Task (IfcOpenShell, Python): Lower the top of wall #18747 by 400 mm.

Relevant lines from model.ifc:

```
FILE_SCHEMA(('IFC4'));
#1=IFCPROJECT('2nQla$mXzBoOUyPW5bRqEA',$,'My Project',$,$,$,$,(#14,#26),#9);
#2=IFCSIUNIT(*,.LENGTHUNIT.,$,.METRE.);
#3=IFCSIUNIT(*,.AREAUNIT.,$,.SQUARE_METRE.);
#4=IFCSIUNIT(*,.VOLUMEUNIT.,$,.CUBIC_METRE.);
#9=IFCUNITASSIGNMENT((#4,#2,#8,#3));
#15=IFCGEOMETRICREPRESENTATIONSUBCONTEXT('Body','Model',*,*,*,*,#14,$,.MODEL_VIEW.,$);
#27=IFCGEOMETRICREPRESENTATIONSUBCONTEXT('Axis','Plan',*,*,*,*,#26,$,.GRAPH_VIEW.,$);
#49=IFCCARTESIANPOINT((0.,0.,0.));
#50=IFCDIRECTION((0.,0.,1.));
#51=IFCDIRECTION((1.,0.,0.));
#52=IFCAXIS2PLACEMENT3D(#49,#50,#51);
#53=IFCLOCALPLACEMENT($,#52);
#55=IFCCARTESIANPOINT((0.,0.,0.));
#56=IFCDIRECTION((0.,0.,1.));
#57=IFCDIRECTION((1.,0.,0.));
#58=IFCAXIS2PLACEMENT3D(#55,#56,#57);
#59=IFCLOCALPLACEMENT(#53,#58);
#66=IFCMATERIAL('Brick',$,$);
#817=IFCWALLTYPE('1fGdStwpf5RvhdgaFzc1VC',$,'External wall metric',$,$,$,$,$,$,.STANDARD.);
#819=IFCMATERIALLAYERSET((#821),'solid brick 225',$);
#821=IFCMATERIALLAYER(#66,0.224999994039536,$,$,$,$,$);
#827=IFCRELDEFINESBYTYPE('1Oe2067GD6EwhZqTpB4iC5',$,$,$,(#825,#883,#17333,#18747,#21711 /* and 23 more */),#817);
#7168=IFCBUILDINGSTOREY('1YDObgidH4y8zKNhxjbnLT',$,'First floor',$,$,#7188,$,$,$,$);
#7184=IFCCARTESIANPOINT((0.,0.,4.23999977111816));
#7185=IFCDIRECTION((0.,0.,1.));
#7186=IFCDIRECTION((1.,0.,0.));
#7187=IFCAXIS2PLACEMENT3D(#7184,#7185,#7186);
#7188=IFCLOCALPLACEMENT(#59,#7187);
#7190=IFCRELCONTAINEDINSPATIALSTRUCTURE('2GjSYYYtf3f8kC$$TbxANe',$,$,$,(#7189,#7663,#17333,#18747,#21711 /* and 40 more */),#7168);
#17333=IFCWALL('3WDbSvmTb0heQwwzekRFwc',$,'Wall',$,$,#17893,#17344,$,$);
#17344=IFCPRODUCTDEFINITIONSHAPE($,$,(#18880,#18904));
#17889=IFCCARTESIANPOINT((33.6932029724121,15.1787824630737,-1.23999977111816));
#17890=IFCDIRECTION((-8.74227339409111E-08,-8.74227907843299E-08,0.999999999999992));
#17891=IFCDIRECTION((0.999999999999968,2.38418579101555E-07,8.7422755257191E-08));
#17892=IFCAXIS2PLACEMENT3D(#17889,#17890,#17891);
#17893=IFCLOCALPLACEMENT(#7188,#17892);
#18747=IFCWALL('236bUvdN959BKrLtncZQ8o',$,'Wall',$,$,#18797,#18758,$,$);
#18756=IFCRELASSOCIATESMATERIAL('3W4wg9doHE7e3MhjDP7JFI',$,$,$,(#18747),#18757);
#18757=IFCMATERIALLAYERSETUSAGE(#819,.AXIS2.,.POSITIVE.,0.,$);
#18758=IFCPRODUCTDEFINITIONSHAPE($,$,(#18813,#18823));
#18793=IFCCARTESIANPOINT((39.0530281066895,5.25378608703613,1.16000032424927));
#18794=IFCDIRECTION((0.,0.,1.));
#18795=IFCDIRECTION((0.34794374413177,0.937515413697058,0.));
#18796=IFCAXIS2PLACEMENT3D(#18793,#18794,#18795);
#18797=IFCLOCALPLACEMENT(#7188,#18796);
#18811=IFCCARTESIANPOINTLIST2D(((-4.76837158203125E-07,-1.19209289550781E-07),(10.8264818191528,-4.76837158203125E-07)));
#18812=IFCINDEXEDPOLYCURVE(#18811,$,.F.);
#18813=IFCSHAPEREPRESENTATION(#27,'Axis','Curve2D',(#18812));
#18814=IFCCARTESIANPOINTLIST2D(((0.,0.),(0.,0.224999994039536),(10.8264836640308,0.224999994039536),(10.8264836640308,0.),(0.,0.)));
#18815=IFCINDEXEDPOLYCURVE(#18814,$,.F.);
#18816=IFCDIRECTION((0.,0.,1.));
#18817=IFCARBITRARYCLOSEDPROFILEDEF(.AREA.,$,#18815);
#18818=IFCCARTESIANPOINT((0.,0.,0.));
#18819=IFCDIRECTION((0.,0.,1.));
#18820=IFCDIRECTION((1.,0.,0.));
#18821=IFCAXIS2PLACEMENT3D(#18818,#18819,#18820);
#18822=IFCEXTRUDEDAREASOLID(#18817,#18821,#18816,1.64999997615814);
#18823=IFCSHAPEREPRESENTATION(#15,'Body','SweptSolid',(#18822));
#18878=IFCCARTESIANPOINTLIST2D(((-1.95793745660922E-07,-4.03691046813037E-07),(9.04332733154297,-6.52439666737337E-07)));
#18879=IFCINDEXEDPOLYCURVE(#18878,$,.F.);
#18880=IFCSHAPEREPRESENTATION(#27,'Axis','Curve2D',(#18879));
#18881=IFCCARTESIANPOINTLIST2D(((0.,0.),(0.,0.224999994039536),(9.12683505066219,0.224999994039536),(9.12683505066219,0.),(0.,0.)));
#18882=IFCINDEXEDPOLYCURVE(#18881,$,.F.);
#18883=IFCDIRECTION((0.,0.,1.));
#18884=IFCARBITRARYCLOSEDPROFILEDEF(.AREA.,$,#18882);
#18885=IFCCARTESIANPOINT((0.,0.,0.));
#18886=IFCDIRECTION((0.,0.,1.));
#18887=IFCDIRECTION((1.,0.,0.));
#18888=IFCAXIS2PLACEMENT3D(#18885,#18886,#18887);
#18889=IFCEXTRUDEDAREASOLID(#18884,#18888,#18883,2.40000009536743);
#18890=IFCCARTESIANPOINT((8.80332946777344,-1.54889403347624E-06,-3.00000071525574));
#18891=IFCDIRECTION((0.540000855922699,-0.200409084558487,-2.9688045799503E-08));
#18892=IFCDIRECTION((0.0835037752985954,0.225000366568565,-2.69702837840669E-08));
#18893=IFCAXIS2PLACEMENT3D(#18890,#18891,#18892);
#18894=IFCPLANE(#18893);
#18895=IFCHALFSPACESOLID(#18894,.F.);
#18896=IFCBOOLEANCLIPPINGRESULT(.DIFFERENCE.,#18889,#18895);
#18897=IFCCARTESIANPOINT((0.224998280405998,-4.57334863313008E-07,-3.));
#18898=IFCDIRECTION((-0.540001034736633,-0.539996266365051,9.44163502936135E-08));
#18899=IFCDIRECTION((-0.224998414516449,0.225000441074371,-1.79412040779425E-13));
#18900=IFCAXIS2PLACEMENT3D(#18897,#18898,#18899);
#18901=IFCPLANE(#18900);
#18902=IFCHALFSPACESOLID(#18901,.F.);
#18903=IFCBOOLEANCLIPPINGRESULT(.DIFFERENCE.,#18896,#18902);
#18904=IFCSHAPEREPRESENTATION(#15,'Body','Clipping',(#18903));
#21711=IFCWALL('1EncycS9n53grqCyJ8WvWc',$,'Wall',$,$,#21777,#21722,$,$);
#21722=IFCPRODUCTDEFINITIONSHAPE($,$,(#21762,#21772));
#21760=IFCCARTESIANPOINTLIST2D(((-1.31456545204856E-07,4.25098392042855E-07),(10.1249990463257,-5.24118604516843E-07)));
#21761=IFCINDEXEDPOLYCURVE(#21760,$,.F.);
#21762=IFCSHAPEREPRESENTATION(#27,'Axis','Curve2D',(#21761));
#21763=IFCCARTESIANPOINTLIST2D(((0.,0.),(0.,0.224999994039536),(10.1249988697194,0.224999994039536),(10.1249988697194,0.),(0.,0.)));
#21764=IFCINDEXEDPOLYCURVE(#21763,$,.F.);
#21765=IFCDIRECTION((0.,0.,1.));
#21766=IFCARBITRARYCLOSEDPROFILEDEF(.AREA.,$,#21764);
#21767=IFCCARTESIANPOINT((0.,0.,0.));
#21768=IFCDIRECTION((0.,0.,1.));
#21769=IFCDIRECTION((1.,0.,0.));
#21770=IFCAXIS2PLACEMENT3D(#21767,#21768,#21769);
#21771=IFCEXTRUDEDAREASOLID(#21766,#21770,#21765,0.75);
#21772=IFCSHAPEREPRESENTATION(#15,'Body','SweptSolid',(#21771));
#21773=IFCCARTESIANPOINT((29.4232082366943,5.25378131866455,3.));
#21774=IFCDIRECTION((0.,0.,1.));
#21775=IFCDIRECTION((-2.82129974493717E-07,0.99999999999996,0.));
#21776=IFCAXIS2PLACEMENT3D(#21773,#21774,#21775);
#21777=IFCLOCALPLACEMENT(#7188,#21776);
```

```python
import ifcopenshell
import ifcopenshell.geom
import ifcopenshell.util.representation
import ifcopenshell.util.shape
import ifcopenshell.util.unit

model = ifcopenshell.open("model.ifc")
unit_scale = ifcopenshell.util.unit.calculate_unit_scale(model)
settings = ifcopenshell.geom.settings()


def volume(element):
    """Net volume in cubic metres, openings subtracted."""
    shape = ifcopenshell.geom.create_shape(settings, element)
    return ifcopenshell.util.shape.get_volume(shape.geometry)


wall = model.by_guid("236bUvdN959BKrLtncZQ8o")
before = volume(wall)

body = ifcopenshell.util.representation.get_representation(wall, "Model", "Body")
solid = body.Items[0]
old_height = solid.Depth
solid.Depth -= 0.4 / unit_scale
after = volume(wall)

print(f"height {old_height:g} -> {solid.Depth:g}, volume {before:.3f} -> {after:.3f} m3")

model.write("model-out.ifc")
```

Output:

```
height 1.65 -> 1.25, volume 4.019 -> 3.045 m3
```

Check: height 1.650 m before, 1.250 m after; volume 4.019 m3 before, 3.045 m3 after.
